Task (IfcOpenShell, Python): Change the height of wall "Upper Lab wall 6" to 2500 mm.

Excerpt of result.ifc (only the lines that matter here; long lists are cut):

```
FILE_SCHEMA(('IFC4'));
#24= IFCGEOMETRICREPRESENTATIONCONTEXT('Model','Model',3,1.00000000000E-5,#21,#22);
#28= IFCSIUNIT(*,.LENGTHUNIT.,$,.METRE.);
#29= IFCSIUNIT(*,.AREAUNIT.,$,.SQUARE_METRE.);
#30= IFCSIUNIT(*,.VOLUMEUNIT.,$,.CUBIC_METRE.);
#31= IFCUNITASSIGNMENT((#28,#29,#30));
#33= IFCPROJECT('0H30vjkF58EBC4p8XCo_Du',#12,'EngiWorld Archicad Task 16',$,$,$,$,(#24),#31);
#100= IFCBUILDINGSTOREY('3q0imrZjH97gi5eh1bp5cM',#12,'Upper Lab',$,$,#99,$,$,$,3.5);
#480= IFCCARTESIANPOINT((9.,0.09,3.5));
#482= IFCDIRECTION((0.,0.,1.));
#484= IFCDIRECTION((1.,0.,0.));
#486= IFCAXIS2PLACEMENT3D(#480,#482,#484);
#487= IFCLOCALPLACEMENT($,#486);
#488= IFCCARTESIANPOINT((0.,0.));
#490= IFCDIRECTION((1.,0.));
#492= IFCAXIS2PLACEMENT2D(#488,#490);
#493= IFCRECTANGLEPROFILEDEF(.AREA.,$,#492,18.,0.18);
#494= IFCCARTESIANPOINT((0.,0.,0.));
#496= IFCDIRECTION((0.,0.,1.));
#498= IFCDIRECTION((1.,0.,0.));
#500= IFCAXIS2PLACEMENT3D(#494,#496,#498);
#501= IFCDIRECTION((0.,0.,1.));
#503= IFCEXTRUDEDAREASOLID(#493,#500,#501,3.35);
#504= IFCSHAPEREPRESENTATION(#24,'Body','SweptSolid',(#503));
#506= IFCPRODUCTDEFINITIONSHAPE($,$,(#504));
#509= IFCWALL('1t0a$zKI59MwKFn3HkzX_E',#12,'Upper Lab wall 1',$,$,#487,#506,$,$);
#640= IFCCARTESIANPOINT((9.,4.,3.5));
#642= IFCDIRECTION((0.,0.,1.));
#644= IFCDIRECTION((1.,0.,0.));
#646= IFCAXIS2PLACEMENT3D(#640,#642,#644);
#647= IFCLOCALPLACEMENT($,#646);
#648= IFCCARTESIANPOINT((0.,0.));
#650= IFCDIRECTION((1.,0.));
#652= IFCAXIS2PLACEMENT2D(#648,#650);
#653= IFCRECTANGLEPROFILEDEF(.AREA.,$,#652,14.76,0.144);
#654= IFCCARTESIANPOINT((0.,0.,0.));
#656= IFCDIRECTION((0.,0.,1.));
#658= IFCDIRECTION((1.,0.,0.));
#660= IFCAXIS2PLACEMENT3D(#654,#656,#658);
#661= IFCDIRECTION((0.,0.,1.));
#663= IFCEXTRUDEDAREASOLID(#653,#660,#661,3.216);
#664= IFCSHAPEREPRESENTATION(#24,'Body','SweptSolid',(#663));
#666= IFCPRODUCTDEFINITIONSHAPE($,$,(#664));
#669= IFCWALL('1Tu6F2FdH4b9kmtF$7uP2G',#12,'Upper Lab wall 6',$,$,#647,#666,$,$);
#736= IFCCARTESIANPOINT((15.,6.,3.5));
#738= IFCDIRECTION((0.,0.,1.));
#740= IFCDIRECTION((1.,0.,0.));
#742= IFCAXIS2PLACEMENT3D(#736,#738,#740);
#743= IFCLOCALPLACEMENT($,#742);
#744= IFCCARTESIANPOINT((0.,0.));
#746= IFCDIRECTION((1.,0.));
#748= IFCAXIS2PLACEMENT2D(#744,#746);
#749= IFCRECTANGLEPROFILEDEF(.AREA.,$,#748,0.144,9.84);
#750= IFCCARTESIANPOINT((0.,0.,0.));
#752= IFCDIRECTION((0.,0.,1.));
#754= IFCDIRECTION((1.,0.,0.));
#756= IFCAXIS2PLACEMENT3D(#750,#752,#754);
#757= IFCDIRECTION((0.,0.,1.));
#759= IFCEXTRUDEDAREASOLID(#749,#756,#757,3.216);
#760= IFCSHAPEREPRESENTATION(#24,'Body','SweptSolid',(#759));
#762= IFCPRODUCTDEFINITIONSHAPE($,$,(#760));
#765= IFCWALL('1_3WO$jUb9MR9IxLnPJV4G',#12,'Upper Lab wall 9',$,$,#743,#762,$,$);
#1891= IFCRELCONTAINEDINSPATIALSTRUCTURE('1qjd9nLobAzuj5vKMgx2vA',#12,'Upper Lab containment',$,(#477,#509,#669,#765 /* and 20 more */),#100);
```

```python
import ifcopenshell
import ifcopenshell.geom
import ifcopenshell.util.shape
import ifcopenshell.util.unit

model = ifcopenshell.open("result.ifc")
unit_scale = ifcopenshell.util.unit.calculate_unit_scale(model)
settings = ifcopenshell.geom.settings()


def volume(element):
    """Net volume in cubic metres, openings subtracted."""
    shape = ifcopenshell.geom.create_shape(settings, element)
    return ifcopenshell.util.shape.get_volume(shape.geometry)


wall = model.by_id(669)
before = volume(wall)

body = next(r for r in wall.Representation.Representations if r.RepresentationIdentifier == "Body")
solid = body.Items[0]
old_height = solid.Depth
solid.Depth = 2.5 / unit_scale
after = volume(wall)

print(f"height {old_height:g} -> {solid.Depth:g}, volume {before:.3f} -> {after:.3f} m3")

model.write("result_v2.ifc")
```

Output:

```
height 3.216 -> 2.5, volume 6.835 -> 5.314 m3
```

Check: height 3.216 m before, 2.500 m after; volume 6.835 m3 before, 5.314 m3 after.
